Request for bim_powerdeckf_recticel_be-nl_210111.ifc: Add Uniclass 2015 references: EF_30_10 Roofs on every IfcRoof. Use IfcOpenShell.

First a look at what the model holds.

```python
import ifcopenshell

model = ifcopenshell.open("bim_powerdeckf_recticel_be-nl_210111.ifc")
print(model.schema)
print("classifications:", [c.Name for c in model.by_type("IfcClassification")])
for ifc_class in ("IfcDoor", "IfcRoof", "IfcStair", "IfcWall", "IfcWindow"):
    print(ifc_class, len(model.by_type(ifc_class)))
```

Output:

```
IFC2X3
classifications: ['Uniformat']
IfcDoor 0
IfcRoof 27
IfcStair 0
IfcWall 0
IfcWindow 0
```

```python
import ifcopenshell
import ifcopenshell.api.classification

model = ifcopenshell.open("bim_powerdeckf_recticel_be-nl_210111.ifc")

# IFC2X3 requires Source and Edition and has no link from the project to the system.
system = model.create_entity("IfcClassification", Source="NBS", Edition="2015", Name="Uniclass 2015")

codes = {
    "IfcRoof": ("EF_30_10", "Roofs"),
}
for ifc_class, (code, name) in codes.items():
    products = model.by_type(ifc_class)
    ifcopenshell.api.classification.add_reference(
        model, products=products, classification=system, identification=code, name=name
    )
    print(code, len(products))

model.write("bim_powerdeckf_recticel_be-nl_210111_updated.ifc")
```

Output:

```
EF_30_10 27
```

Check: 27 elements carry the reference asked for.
